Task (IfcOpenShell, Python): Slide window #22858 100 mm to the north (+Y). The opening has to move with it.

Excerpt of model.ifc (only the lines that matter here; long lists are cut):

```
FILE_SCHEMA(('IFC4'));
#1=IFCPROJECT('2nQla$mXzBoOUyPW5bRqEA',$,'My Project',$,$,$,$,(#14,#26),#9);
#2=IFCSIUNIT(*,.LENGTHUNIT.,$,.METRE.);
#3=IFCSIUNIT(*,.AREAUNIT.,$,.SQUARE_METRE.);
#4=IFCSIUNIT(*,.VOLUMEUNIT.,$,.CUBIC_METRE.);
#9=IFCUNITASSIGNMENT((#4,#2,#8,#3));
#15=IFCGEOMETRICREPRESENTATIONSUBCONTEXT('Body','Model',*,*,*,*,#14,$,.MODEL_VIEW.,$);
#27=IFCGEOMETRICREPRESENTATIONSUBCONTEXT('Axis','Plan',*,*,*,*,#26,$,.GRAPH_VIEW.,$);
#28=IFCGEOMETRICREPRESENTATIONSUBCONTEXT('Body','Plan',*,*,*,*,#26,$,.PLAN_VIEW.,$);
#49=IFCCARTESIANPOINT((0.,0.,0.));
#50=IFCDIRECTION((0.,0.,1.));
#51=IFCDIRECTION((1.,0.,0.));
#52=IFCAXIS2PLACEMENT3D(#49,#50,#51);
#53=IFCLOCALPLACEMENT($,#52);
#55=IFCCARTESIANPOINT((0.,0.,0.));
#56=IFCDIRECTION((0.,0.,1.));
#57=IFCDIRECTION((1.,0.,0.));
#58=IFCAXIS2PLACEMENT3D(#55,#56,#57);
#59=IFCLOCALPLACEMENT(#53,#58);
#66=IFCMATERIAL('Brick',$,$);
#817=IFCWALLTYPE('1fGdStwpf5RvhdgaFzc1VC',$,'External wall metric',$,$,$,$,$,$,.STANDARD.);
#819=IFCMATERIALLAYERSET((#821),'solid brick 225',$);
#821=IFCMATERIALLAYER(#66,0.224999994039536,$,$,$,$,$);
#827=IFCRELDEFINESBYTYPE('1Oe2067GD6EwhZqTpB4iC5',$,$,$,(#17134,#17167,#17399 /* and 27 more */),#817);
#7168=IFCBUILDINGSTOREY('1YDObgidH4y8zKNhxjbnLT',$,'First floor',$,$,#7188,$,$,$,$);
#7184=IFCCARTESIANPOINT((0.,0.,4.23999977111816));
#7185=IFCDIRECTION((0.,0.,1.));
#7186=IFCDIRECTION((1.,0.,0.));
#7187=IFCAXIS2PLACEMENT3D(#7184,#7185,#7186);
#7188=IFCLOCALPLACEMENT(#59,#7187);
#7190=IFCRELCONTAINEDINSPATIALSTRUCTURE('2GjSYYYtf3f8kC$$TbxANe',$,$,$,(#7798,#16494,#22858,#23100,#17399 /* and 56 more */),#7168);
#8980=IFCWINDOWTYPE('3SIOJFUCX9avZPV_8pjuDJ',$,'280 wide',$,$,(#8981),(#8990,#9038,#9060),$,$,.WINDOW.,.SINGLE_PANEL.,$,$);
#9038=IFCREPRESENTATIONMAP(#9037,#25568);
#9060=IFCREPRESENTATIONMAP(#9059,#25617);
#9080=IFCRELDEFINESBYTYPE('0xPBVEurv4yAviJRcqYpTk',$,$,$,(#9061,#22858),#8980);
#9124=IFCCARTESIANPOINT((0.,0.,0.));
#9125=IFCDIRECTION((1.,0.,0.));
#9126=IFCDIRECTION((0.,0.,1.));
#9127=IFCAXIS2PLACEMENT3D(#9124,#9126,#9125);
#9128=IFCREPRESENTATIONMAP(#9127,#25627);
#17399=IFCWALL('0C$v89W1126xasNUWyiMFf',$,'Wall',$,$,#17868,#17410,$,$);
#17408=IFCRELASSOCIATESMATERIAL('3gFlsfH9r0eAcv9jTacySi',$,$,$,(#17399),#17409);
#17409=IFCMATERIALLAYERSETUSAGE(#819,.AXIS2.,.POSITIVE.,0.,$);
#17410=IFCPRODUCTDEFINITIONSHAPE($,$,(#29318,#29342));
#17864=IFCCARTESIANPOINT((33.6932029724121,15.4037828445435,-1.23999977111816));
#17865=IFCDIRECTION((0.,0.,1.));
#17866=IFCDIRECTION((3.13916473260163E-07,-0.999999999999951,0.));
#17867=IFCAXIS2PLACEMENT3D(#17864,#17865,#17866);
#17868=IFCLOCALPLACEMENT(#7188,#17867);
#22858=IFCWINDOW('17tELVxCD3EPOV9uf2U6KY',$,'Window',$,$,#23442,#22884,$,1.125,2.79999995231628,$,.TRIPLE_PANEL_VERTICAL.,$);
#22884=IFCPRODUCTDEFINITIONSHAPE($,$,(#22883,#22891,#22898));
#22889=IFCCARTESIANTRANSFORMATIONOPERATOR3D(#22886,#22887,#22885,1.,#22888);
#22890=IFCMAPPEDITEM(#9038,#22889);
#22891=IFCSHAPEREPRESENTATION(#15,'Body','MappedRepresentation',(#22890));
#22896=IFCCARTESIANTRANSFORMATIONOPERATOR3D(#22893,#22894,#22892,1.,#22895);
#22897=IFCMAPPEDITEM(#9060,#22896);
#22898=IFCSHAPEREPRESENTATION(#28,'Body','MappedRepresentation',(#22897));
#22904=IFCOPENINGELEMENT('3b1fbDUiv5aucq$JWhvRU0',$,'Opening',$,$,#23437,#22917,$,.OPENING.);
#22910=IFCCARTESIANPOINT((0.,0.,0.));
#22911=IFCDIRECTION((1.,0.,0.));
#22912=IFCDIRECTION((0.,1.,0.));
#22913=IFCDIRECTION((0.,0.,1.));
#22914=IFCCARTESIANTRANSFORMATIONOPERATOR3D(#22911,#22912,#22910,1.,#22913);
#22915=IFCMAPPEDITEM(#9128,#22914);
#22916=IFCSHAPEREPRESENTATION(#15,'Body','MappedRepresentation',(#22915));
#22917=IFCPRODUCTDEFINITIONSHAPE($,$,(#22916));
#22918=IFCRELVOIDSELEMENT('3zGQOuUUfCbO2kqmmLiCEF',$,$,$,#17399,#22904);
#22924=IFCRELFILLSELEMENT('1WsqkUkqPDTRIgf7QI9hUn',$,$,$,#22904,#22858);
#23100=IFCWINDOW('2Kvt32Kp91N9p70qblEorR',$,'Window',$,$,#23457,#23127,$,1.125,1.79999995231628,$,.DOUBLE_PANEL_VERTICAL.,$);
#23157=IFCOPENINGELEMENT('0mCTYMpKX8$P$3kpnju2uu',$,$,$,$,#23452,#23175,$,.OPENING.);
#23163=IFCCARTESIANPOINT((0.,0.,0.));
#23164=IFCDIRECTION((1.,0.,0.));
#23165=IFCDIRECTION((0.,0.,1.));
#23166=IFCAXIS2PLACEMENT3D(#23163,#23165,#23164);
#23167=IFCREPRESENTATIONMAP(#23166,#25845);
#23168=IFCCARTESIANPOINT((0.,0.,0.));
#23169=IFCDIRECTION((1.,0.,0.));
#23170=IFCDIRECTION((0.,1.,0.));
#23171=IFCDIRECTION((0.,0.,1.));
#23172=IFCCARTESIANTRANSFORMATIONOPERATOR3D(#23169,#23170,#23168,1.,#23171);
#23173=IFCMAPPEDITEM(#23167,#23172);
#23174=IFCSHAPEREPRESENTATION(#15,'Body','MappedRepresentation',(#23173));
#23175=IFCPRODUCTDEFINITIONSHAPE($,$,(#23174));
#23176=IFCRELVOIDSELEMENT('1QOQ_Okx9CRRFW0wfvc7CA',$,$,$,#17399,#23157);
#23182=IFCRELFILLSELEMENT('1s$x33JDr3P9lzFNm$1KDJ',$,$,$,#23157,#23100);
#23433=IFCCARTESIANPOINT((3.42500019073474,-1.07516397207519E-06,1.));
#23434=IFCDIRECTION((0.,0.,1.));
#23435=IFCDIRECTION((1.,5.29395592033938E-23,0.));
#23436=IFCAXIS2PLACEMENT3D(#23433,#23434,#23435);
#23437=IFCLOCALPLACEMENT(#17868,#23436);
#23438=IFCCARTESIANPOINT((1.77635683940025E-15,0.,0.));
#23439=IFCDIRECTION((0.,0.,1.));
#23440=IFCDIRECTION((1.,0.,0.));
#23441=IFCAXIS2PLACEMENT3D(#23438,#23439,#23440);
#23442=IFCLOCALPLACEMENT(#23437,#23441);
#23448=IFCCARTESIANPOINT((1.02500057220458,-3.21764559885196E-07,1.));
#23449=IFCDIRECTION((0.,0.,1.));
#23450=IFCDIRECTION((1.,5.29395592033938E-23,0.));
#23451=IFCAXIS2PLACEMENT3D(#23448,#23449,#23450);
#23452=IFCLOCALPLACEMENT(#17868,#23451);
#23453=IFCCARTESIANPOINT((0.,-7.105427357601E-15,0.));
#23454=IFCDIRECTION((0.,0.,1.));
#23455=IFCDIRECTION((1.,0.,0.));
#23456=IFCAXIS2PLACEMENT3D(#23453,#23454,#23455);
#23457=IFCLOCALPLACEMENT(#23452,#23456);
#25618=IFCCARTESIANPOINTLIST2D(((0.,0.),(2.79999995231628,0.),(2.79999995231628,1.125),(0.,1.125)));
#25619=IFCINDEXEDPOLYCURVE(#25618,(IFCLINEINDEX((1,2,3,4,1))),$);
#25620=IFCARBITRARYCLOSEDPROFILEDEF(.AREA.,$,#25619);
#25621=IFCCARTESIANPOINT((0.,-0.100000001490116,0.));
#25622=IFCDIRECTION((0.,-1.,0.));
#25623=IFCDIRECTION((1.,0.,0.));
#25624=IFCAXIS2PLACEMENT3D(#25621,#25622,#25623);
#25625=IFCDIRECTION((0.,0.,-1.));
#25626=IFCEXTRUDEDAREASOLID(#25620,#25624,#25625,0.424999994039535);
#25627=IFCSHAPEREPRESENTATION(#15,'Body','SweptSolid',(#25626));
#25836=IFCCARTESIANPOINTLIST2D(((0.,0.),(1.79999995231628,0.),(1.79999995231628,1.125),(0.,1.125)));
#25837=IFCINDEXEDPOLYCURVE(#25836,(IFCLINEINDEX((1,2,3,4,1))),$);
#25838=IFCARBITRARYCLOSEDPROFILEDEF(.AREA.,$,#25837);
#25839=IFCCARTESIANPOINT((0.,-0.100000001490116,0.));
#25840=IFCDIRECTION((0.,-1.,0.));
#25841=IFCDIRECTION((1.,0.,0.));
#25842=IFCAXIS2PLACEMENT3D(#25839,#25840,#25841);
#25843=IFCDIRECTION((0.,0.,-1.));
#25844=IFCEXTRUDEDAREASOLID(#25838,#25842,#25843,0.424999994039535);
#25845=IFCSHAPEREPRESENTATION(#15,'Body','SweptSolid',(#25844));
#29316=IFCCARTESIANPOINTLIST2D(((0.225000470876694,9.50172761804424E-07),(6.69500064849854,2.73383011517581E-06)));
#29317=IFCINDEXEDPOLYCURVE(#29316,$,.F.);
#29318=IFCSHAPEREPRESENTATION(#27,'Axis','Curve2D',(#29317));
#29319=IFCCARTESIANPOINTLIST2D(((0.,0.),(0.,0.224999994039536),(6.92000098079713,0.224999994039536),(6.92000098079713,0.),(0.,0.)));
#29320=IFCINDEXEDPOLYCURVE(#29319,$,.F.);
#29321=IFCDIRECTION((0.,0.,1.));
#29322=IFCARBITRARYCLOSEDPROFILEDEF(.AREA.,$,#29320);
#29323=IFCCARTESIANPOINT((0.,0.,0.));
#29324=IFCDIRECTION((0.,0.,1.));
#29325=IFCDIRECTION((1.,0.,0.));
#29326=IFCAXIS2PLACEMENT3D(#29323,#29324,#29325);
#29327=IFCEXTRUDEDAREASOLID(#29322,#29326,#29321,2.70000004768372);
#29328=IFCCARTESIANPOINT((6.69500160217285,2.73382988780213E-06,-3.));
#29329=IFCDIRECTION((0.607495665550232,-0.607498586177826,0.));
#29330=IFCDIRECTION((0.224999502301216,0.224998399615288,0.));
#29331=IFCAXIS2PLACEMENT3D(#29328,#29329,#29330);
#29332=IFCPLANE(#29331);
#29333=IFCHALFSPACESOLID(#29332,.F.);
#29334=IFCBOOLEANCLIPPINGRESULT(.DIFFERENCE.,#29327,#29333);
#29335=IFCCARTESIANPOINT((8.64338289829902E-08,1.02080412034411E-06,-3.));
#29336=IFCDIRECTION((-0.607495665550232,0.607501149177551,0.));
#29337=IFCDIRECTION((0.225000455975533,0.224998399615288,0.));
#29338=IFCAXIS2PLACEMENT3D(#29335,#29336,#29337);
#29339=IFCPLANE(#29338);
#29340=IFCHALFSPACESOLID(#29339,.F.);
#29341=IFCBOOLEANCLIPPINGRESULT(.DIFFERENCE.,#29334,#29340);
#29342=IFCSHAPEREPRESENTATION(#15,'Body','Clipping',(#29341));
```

```python
import ifcopenshell
import ifcopenshell.api.geometry
import ifcopenshell.util.placement

model = ifcopenshell.open("model.ifc")

window = model.by_guid("17tELVxCD3EPOV9uf2U6KY")
opening = window.FillsVoids[0].RelatingOpeningElement
wall = opening.VoidsElements[0].RelatingBuildingElement

wall_matrix = ifcopenshell.util.placement.get_local_placement(wall.ObjectPlacement)
shift = wall_matrix[:3, 0] * -0.1
before = ifcopenshell.util.placement.get_local_placement(window.ObjectPlacement)[:3, 3].copy()

# The window is placed relative to its opening, so it follows when the opening moves.
matrix = ifcopenshell.util.placement.get_local_placement(opening.ObjectPlacement)
matrix[:3, 3] += shift
ifcopenshell.api.geometry.edit_object_placement(
    model, product=opening, matrix=matrix, is_si=False, should_transform_children=True
)

after = ifcopenshell.util.placement.get_local_placement(window.ObjectPlacement)[:3, 3]
print("window moved by", (after - before).round(3) + 0.0)

model.write("model_v2.ifc")
```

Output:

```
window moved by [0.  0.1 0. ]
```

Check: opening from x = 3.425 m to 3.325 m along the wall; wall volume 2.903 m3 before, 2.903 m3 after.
